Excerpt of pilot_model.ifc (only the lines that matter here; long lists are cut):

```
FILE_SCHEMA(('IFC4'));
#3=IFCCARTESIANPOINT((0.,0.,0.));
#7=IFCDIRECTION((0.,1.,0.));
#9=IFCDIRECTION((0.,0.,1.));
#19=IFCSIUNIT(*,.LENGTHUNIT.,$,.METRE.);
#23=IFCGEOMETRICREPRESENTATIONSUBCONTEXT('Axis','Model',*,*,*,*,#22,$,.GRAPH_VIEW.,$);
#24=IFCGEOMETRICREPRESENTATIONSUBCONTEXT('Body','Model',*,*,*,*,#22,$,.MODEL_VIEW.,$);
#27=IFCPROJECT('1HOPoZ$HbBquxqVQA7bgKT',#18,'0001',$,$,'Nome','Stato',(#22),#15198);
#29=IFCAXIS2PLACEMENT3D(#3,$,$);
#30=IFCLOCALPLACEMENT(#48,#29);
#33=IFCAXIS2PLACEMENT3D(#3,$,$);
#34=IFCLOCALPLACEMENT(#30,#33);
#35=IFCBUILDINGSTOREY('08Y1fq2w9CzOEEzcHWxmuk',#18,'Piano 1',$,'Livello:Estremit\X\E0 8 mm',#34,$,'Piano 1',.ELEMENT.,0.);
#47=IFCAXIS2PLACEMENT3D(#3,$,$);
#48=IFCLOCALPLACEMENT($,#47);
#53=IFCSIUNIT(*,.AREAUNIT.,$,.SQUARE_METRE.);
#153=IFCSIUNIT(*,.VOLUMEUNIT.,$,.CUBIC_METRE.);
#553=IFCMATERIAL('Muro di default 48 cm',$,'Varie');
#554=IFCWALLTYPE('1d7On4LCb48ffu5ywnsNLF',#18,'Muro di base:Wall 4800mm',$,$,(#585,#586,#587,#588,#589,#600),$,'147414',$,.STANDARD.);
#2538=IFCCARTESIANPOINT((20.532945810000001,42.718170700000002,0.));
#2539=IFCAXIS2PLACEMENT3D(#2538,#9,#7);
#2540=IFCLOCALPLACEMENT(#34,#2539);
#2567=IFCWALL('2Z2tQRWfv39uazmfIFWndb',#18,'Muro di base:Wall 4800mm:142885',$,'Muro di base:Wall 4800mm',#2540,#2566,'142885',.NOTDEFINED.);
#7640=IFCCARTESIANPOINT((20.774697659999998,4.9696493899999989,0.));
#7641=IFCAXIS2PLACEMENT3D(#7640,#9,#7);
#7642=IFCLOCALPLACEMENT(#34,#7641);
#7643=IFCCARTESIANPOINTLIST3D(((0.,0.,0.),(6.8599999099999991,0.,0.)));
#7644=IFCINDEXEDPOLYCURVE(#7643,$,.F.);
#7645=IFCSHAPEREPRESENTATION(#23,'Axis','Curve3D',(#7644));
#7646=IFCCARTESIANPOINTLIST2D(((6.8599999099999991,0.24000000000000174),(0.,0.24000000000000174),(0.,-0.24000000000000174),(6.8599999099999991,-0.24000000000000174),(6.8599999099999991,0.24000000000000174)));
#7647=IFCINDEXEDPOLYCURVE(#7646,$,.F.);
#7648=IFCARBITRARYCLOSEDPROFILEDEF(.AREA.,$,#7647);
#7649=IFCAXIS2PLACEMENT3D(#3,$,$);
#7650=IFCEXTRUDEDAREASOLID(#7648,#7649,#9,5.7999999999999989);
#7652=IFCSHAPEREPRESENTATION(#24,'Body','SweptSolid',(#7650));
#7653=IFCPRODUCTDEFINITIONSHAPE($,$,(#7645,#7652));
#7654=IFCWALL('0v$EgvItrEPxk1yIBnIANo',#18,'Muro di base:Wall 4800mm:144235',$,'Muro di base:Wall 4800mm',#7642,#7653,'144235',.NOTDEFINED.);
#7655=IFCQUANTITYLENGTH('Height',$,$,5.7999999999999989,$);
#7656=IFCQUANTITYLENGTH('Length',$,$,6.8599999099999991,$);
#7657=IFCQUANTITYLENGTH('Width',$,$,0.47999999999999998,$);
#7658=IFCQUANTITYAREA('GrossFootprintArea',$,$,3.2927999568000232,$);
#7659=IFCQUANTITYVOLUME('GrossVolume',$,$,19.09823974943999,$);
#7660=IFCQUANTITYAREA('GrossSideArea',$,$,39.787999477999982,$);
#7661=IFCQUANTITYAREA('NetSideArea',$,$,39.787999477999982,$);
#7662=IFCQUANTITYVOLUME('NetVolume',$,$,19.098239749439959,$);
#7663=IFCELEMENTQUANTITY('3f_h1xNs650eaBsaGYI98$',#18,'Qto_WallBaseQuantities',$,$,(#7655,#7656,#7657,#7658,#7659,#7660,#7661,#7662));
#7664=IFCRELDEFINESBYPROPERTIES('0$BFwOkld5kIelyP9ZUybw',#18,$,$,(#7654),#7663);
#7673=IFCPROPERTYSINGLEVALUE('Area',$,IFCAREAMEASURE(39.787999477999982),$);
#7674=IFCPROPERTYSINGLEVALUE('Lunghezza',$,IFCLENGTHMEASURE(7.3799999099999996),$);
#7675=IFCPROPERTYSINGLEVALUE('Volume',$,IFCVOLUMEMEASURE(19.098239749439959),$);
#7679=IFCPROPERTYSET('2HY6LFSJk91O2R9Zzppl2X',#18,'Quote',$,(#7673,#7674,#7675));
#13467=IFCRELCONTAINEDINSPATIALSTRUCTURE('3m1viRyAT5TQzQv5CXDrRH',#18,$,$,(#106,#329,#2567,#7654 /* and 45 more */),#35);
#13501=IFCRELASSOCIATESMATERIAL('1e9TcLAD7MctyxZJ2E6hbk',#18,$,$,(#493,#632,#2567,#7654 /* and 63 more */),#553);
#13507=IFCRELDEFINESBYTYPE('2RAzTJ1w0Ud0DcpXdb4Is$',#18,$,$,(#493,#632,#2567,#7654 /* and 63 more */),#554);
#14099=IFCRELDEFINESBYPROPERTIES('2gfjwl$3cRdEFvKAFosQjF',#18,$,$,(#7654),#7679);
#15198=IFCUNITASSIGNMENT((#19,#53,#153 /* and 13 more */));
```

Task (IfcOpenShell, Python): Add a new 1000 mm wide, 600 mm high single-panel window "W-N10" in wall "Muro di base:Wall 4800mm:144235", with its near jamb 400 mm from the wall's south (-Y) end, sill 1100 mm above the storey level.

```python
import numpy as np
import ifcopenshell
import ifcopenshell.api.feature
import ifcopenshell.api.geometry
import ifcopenshell.api.pset
import ifcopenshell.api.root
import ifcopenshell.api.spatial
import ifcopenshell.geom
import ifcopenshell.util.element
import ifcopenshell.util.placement
import ifcopenshell.util.representation
import ifcopenshell.util.shape
import ifcopenshell.util.unit

model = ifcopenshell.open("pilot_model.ifc")
unit_scale = ifcopenshell.util.unit.calculate_unit_scale(model)
area_scale = ifcopenshell.util.unit.calculate_unit_scale(model, "AREAUNIT")
volume_scale = ifcopenshell.util.unit.calculate_unit_scale(model, "VOLUMEUNIT")
settings = ifcopenshell.geom.settings()


def volume(element):
    """Net volume in cubic metres, openings subtracted."""
    shape = ifcopenshell.geom.create_shape(settings, element)
    return ifcopenshell.util.shape.get_volume(shape.geometry)


wall = model.by_guid("0v$EgvItrEPxk1yIBnIANo")
storey = ifcopenshell.util.element.get_container(wall, ifc_class="IfcBuildingStorey")
context = ifcopenshell.util.representation.get_context(model, "Model", "Body", "MODEL_VIEW")
before = volume(wall)

width, height, from_end, sill = 1, 0.6, 0.4, 1.1  # metres

# The wall runs along its own X axis, and the end named is its -X end.
wall_shape = ifcopenshell.geom.create_shape(settings, wall)
x, y, z = ifcopenshell.util.shape.get_vertices(wall_shape.geometry).T
start = x.min() + from_end
face, thickness = float(y.min()), float(y.max() - y.min())
wall_matrix = ifcopenshell.util.placement.get_local_placement(wall.ObjectPlacement)
level = ifcopenshell.util.placement.get_local_placement(storey.ObjectPlacement)[2, 3]


def in_wall(x, y):
    """Placement at x, y metres in the wall's axes, at sill height."""
    matrix = wall_matrix.copy()
    matrix[:, 3] = wall_matrix @ np.array([x / unit_scale, y / unit_scale, 0.0, 1.0])
    matrix[2, 3] = level + sill / unit_scale
    return matrix


# Opening: a box that overshoots both wall faces by 50 mm.
opening = ifcopenshell.api.root.create_entity(model, ifc_class="IfcOpeningElement", predefined_type="OPENING")
box = ifcopenshell.api.geometry.add_wall_representation(
    model, context=context, length=width, height=height, thickness=thickness + 0.1
)
ifcopenshell.api.geometry.assign_representation(model, product=opening, representation=box)
ifcopenshell.api.geometry.edit_object_placement(model, product=opening, matrix=in_wall(start, face - 0.05), is_si=False)
ifcopenshell.api.feature.add_feature(model, feature=opening, element=wall)

window = ifcopenshell.api.root.create_entity(model, ifc_class="IfcWindow", name="W-N10", predefined_type="WINDOW")
window.OverallWidth, window.OverallHeight = width / unit_scale, height / unit_scale
window.PartitioningType = "SINGLE_PANEL"
body = ifcopenshell.api.geometry.add_window_representation(
    model,
    context=context,
    overall_width=window.OverallWidth,
    overall_height=window.OverallHeight,
    partition_type="SINGLE_PANEL",
)
ifcopenshell.api.geometry.assign_representation(model, product=window, representation=body)
ifcopenshell.api.spatial.assign_container(model, products=[window], relating_structure=storey)
ifcopenshell.api.feature.add_filling(model, opening=opening, element=window)

# Centre the window in the wall's thickness.
ifcopenshell.api.geometry.edit_object_placement(model, product=window, matrix=in_wall(start, face), is_si=False)
window_shape = ifcopenshell.geom.create_shape(settings, window)
depth = ifcopenshell.util.shape.get_vertices(window_shape.geometry)[:, 1]
offset = face + thickness / 2 - (depth.min() + depth.max()) / 2
ifcopenshell.api.geometry.edit_object_placement(model, product=window, matrix=in_wall(start, offset), is_si=False)

after = volume(wall)

# Update the wall's stored quantities.
qto = model.by_id(ifcopenshell.util.element.get_pset(wall, "Qto_WallBaseQuantities", should_inherit=False)["id"])
ifcopenshell.api.pset.edit_qto(model, qto=qto, properties={
    "NetSideArea": after / thickness / area_scale,
    "NetVolume": after / volume_scale,
})
pset = model.by_id(ifcopenshell.util.element.get_pset(wall, "Quote", should_inherit=False)["id"])
ifcopenshell.api.pset.edit_pset(model, pset=pset, properties={
    "Area": model.create_entity("IfcAreaMeasure", after / thickness / area_scale),
    "Volume": model.create_entity("IfcVolumeMeasure", after / volume_scale),
})

print(f"wall volume {before:.3f} -> {after:.3f} m3")

model.write("pilot_model_updated.ifc")
```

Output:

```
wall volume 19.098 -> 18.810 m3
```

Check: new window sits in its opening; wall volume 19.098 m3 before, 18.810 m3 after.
